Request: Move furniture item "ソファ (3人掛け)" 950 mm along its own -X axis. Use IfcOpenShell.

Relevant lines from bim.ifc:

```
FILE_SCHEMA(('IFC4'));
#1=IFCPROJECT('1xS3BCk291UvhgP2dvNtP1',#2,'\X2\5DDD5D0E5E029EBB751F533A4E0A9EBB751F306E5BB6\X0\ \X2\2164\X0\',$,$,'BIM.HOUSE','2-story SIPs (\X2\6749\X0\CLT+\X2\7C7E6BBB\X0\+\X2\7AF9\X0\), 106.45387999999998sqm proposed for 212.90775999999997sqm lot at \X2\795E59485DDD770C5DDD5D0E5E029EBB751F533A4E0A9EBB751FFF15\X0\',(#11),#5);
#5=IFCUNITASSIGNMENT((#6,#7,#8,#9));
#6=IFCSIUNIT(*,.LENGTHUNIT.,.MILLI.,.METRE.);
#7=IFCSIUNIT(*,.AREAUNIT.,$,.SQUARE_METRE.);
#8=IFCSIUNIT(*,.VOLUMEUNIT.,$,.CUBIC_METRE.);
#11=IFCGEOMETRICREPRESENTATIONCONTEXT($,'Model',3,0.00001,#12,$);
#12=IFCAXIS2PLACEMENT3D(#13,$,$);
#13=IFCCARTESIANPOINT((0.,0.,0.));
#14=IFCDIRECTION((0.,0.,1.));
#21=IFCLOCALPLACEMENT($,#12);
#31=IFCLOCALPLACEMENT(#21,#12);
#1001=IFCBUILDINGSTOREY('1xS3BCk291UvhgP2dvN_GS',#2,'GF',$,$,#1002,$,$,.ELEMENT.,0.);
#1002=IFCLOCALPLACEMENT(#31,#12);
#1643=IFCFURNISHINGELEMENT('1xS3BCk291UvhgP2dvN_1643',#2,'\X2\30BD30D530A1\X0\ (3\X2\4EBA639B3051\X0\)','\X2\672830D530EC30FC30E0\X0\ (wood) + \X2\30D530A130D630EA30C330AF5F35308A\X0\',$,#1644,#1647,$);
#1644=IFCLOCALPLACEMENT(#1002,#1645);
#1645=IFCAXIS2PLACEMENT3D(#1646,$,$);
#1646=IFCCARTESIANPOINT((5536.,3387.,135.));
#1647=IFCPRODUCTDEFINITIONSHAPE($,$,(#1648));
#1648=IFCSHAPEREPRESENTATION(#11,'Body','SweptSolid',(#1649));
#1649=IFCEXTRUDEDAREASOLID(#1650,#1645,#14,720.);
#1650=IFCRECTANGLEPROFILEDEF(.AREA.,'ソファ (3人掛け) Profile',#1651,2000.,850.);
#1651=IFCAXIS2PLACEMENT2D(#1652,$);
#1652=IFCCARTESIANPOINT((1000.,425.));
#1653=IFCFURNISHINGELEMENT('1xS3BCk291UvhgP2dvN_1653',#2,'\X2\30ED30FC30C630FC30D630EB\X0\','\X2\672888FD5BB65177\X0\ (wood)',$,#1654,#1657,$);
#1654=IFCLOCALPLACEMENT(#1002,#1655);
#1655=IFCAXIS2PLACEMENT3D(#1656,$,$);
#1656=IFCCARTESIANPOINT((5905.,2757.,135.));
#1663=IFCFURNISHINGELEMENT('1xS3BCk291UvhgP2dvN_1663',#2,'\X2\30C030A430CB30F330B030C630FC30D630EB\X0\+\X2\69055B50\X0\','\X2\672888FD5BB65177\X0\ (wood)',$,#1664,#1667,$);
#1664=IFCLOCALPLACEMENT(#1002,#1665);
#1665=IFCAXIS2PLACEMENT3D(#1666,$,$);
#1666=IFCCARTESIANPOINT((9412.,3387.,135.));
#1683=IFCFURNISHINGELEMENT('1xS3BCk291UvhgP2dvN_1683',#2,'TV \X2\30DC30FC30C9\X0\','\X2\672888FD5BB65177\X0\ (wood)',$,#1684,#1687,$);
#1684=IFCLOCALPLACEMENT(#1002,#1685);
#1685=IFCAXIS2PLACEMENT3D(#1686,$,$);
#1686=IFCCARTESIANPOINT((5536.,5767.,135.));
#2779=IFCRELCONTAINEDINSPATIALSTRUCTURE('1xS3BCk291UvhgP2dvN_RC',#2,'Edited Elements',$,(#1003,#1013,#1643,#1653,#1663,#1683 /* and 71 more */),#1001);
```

```python
import ifcopenshell
import ifcopenshell.api.geometry
import ifcopenshell.util.placement
import ifcopenshell.util.unit

model = ifcopenshell.open("bim.ifc")
unit_scale = ifcopenshell.util.unit.calculate_unit_scale(model)

item = model.by_guid("1xS3BCk291UvhgP2dvN_1643")
matrix = ifcopenshell.util.placement.get_local_placement(item.ObjectPlacement)
matrix[:3, 3] -= matrix[:3, 0] * 0.95 / unit_scale
ifcopenshell.api.geometry.edit_object_placement(model, product=item, matrix=matrix, is_si=False)

print(ifcopenshell.util.placement.get_local_placement(item.ObjectPlacement).round(3) + 0.0)

model.write("bim_edited.ifc")
```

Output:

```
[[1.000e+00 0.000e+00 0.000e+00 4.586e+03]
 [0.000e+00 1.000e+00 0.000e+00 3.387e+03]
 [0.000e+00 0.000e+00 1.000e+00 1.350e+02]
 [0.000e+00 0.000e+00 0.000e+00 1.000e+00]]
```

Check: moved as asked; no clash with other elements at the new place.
